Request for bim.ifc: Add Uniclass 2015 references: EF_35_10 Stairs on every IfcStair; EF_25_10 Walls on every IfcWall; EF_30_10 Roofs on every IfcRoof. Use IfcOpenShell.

First a look at what the model holds.

```python
import ifcopenshell

model = ifcopenshell.open("bim.ifc")
print(model.schema)
print("classifications:", [c.Name for c in model.by_type("IfcClassification")])
for ifc_class in ("IfcDoor", "IfcRoof", "IfcStair", "IfcWall", "IfcWindow"):
    print(ifc_class, len(model.by_type(ifc_class)))
```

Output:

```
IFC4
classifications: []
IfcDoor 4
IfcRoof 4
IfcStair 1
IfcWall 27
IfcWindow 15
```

```python
import ifcopenshell
import ifcopenshell.api.classification

model = ifcopenshell.open("bim.ifc")

system = ifcopenshell.api.classification.add_classification(model, classification="Uniclass 2015")

codes = {
    "IfcStair": ("EF_35_10", "Stairs"),
    "IfcWall": ("EF_25_10", "Walls"),
    "IfcRoof": ("EF_30_10", "Roofs"),
}
for ifc_class, (code, name) in codes.items():
    products = model.by_type(ifc_class)
    ifcopenshell.api.classification.add_reference(
        model, products=products, classification=system, identification=code, name=name
    )
    print(code, len(products))

model.write("bim-out.ifc")
```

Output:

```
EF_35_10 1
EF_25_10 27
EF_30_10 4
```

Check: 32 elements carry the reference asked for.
